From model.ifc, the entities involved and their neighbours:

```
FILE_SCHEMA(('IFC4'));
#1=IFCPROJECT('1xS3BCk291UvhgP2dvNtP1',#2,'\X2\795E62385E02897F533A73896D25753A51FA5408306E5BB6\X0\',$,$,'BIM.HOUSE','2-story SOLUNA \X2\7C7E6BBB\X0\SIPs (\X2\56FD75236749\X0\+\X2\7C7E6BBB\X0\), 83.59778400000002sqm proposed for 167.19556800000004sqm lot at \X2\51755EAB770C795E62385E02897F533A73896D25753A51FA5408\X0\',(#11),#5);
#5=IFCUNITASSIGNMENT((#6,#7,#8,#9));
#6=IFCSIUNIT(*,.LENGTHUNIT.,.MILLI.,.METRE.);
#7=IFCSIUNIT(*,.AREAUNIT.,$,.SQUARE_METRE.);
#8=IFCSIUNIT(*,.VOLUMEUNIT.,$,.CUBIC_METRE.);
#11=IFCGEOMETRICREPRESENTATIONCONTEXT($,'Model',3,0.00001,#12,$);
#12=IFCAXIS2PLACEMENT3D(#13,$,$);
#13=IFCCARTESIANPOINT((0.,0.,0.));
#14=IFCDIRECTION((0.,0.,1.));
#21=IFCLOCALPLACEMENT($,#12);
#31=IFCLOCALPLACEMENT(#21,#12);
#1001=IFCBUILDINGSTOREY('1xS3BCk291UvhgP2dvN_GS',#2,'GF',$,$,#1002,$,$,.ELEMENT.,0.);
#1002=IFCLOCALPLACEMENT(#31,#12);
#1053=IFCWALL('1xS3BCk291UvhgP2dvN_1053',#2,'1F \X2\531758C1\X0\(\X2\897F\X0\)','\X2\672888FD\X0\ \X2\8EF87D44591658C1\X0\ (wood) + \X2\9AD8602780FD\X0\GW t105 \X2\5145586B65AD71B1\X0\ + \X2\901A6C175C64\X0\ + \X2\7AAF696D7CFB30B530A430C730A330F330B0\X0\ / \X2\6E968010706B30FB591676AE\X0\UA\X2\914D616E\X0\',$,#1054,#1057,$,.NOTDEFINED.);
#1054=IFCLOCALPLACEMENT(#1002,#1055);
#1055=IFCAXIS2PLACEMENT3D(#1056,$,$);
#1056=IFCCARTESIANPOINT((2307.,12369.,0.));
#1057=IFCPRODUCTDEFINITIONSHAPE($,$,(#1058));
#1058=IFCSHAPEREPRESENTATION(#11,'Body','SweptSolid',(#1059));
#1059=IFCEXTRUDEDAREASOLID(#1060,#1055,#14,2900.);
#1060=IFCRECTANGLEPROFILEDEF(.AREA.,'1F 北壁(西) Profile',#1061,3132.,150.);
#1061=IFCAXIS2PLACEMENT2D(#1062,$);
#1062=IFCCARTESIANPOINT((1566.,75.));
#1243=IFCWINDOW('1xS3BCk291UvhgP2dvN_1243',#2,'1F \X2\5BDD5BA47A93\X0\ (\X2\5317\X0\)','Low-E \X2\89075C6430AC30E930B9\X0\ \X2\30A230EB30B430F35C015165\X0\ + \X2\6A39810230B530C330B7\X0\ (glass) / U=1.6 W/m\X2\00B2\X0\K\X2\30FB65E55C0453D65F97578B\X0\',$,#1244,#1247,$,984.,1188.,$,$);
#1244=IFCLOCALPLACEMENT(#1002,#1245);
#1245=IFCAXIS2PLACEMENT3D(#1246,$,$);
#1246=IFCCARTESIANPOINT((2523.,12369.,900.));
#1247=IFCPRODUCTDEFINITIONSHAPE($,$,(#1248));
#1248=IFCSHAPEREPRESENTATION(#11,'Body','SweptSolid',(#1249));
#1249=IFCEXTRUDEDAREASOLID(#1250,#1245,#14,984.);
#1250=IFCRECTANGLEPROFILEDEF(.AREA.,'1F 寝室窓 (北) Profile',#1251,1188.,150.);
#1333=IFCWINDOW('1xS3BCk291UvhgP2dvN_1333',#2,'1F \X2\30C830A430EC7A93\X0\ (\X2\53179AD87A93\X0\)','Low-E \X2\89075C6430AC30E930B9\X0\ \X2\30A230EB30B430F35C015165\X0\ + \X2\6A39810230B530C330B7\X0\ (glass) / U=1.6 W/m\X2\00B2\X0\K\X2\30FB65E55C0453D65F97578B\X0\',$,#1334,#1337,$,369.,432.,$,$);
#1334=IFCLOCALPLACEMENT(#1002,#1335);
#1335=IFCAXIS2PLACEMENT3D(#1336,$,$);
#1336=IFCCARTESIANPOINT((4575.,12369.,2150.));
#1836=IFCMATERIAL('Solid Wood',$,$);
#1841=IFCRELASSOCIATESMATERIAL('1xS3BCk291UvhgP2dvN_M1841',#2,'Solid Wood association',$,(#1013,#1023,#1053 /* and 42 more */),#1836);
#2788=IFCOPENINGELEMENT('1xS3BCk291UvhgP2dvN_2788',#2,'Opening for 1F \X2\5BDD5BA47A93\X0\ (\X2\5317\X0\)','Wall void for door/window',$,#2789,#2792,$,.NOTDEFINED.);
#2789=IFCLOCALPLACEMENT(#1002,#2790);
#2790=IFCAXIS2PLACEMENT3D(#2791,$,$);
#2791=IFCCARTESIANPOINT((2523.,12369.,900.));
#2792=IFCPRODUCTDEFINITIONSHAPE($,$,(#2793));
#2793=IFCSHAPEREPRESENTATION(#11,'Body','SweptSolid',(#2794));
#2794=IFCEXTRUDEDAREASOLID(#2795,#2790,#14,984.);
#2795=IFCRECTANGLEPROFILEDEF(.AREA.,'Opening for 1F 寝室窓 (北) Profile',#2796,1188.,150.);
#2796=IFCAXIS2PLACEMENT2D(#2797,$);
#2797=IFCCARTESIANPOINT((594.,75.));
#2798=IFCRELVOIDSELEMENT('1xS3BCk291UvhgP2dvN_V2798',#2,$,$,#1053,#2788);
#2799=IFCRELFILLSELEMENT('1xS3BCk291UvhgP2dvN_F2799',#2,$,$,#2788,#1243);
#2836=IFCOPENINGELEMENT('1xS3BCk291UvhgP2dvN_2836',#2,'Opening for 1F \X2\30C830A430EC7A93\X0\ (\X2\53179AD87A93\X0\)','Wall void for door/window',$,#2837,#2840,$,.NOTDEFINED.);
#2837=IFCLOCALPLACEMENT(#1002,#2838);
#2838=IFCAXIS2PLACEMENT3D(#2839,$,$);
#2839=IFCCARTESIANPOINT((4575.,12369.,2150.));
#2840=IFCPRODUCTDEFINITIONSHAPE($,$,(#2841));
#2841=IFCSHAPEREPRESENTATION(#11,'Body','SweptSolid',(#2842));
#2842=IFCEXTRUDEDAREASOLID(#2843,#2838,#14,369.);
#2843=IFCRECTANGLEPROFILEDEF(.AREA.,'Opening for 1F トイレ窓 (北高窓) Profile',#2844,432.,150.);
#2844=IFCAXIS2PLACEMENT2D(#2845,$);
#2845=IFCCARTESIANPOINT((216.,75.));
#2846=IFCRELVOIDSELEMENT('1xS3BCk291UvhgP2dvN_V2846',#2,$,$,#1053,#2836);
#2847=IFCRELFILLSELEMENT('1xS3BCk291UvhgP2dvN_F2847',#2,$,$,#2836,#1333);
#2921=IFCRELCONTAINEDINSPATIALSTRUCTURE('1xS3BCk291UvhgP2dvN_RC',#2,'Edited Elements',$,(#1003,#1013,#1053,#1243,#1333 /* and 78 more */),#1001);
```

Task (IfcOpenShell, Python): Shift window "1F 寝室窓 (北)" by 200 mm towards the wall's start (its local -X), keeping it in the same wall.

```python
import ifcopenshell
import ifcopenshell.api.geometry
import ifcopenshell.util.placement
import ifcopenshell.util.unit

model = ifcopenshell.open("model.ifc")
unit_scale = ifcopenshell.util.unit.calculate_unit_scale(model)

window = model.by_guid("1xS3BCk291UvhgP2dvN_1243")
opening = window.FillsVoids[0].RelatingOpeningElement
wall = opening.VoidsElements[0].RelatingBuildingElement

wall_matrix = ifcopenshell.util.placement.get_local_placement(wall.ObjectPlacement)
shift = wall_matrix[:3, 0] * -0.2 / unit_scale
before = ifcopenshell.util.placement.get_local_placement(window.ObjectPlacement)[:3, 3].copy()

# The window is not placed relative to its opening, so move both.
for product in (opening, window):
    matrix = ifcopenshell.util.placement.get_local_placement(product.ObjectPlacement)
    matrix[:3, 3] += shift
    ifcopenshell.api.geometry.edit_object_placement(model, product=product, matrix=matrix, is_si=False)

after = ifcopenshell.util.placement.get_local_placement(window.ObjectPlacement)[:3, 3]
print("window moved by", (after - before).round(3) + 0.0)

model.write("model_rev.ifc")
```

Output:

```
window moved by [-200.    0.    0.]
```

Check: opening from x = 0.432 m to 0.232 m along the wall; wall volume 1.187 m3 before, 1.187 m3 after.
